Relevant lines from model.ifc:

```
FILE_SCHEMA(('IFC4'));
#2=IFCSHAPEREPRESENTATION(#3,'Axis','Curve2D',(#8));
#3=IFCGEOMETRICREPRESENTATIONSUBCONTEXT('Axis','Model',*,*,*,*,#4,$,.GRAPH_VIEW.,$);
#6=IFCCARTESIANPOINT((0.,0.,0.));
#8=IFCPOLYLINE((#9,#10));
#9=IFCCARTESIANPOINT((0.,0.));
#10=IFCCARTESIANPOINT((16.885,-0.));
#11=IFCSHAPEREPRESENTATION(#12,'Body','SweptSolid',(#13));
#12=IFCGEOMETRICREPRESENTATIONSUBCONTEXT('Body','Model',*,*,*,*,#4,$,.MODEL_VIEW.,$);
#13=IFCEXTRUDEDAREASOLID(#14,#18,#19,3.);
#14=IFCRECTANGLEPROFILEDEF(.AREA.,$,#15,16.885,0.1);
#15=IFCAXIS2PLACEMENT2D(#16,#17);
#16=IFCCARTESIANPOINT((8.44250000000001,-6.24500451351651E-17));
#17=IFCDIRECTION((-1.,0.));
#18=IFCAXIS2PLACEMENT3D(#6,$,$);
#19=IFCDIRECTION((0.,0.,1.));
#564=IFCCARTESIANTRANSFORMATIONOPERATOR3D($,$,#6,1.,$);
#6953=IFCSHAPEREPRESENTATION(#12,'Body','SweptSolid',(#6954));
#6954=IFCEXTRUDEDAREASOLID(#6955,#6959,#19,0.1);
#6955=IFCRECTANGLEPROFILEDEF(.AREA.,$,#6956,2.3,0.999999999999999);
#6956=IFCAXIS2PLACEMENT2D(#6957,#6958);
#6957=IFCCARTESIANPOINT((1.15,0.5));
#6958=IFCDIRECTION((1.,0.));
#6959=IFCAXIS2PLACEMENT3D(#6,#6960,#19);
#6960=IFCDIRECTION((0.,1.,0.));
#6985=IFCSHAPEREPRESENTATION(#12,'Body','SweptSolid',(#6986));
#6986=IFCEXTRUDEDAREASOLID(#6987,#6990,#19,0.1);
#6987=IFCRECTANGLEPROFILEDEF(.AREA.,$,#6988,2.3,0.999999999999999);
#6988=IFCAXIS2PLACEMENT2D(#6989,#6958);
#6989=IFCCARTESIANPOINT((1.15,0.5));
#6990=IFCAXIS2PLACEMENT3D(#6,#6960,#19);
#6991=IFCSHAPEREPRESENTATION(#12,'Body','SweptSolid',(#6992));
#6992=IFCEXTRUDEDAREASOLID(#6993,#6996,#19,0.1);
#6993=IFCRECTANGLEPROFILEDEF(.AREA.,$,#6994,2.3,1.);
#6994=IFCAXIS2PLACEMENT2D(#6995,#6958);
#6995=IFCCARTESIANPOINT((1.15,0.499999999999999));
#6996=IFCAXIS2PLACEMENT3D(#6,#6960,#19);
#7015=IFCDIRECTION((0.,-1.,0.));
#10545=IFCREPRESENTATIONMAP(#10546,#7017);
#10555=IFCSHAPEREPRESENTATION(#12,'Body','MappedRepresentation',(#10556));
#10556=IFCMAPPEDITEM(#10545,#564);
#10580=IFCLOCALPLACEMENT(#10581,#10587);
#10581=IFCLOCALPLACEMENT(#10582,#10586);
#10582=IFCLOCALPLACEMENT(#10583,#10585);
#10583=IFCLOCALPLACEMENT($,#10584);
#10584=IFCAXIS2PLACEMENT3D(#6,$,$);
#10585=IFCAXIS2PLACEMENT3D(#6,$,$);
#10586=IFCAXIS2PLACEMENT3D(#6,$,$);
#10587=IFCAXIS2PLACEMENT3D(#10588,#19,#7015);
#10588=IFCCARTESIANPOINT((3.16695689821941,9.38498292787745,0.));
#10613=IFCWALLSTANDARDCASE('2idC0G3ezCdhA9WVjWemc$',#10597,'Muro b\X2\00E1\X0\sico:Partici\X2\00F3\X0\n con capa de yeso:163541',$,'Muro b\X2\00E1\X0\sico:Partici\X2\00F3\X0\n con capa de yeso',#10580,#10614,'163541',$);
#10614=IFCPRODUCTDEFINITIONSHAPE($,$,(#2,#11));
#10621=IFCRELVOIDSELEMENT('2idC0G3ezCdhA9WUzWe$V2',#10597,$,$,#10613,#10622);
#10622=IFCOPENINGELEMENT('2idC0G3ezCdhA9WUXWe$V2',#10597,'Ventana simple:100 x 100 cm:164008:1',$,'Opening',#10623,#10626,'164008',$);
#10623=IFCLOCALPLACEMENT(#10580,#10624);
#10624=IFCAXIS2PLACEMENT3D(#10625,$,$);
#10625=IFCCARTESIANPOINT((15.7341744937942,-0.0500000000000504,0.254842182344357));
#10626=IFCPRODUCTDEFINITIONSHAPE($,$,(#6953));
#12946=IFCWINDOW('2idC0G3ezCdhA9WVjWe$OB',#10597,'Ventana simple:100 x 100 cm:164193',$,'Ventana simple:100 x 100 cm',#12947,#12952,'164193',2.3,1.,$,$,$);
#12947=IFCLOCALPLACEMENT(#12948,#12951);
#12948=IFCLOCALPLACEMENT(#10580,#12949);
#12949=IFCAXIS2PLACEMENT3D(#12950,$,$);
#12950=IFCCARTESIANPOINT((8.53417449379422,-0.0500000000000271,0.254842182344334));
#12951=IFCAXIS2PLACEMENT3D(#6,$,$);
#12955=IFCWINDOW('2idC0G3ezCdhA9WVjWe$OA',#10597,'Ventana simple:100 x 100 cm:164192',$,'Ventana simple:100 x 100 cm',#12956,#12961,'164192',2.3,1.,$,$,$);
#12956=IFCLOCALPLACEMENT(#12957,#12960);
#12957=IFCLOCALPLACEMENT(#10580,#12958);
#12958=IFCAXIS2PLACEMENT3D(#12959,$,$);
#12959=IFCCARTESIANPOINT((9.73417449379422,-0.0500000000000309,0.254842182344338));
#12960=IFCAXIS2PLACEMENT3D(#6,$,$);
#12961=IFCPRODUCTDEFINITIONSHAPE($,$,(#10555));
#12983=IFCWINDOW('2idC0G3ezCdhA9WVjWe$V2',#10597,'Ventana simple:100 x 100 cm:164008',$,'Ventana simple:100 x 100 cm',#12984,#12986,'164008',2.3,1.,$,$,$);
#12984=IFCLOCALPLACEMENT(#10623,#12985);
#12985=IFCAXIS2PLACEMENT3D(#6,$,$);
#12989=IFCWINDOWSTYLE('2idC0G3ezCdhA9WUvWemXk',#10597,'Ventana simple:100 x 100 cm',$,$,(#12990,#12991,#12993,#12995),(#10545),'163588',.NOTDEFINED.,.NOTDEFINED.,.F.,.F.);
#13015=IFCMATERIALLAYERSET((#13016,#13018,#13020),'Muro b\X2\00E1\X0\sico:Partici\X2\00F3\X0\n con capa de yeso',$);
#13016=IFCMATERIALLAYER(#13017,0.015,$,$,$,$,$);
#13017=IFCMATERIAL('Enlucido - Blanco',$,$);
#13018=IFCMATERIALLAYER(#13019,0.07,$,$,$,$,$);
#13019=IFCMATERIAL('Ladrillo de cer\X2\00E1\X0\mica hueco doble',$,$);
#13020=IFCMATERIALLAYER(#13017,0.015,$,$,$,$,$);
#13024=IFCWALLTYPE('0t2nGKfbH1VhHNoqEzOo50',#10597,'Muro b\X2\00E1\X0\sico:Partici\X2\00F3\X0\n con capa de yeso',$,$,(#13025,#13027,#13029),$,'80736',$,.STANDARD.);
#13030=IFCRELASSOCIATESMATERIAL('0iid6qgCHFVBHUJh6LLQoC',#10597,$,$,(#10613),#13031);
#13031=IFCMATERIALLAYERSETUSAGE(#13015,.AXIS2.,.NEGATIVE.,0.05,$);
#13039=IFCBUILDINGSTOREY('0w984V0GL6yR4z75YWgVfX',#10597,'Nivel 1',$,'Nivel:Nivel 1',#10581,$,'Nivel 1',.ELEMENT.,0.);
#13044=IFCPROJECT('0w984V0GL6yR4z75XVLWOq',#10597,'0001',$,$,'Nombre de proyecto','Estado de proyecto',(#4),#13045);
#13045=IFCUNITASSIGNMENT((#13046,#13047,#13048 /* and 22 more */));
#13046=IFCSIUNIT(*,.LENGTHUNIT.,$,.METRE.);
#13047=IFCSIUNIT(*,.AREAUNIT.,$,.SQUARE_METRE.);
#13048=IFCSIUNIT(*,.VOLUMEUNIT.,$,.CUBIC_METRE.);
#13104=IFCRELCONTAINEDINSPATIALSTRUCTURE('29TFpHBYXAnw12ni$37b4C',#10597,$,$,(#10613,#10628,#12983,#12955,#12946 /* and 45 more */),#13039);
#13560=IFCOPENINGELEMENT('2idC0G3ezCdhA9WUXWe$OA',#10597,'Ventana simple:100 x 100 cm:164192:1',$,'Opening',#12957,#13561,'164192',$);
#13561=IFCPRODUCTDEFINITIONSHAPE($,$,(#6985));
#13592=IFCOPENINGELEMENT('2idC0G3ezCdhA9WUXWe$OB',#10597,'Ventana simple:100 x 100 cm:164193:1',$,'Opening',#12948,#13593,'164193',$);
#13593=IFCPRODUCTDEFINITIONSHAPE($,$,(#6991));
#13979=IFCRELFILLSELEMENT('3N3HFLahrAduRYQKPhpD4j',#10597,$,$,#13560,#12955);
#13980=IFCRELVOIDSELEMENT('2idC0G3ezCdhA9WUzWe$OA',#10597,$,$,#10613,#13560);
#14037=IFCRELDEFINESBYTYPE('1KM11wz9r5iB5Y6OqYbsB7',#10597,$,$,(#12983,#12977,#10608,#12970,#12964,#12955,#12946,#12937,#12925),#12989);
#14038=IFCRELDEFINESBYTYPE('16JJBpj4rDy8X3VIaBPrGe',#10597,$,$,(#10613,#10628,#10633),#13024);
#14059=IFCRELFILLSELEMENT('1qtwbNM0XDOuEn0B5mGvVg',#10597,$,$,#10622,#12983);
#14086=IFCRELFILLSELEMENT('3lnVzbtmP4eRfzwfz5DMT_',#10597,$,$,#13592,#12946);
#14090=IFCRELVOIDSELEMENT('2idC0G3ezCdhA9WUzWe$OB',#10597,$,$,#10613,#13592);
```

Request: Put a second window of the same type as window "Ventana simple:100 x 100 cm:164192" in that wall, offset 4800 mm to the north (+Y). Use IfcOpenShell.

```python
import ifcopenshell
import ifcopenshell.api.feature
import ifcopenshell.api.geometry
import ifcopenshell.api.root
import ifcopenshell.geom
import ifcopenshell.util.element
import ifcopenshell.util.placement
import ifcopenshell.util.shape

model = ifcopenshell.open("model.ifc")
settings = ifcopenshell.geom.settings()


def volume(element):
    """Net volume in cubic metres, openings subtracted."""
    shape = ifcopenshell.geom.create_shape(settings, element)
    return ifcopenshell.util.shape.get_volume(shape.geometry)


def reuse_history(source, copy):
    """copy_class also copies each property set's owner history, people and application; keep the originals."""
    for rel in copy.IsDefinedBy:
        if rel.is_a("IfcRelDefinesByProperties") and (history := rel.RelatingPropertyDefinition.OwnerHistory):
            rel.RelatingPropertyDefinition.OwnerHistory = source.OwnerHistory
            ifcopenshell.util.element.remove_deep2(model, history)


window = model.by_guid("2idC0G3ezCdhA9WVjWe$OA")
opening = window.FillsVoids[0].RelatingOpeningElement
wall = opening.VoidsElements[0].RelatingBuildingElement
before = volume(wall)
shift = ifcopenshell.util.placement.get_local_placement(wall.ObjectPlacement)[:3, 0] * -4.8

# copy_class copies the void relationship, type, container and properties, but no geometry.
new_opening = ifcopenshell.api.root.copy_class(model, product=opening)
new_opening.Representation = ifcopenshell.util.element.copy_deep(
    model, opening.Representation, exclude=["IfcGeometricRepresentationContext", "IfcRepresentationMap"]
)
new_opening.Name = "Ventana simple:100 x 100 cm"
new_opening.Tag = None
new_window = ifcopenshell.api.root.copy_class(model, product=window)
new_window.Representation = ifcopenshell.util.element.copy_deep(
    model, window.Representation, exclude=["IfcGeometricRepresentationContext", "IfcRepresentationMap"]
)
new_window.Name = "Ventana simple:100 x 100 cm"
new_window.Tag = None
reuse_history(window, new_window)
ifcopenshell.api.feature.add_filling(model, opening=new_opening, element=new_window)

for old, new in ((opening, new_opening), (window, new_window)):
    matrix = ifcopenshell.util.placement.get_local_placement(old.ObjectPlacement)
    matrix[:3, 3] += shift
    ifcopenshell.api.geometry.edit_object_placement(model, product=new, matrix=matrix, is_si=False)

after = volume(wall)

print(f"wall volume {before:.3f} -> {after:.3f} m3")

model.write("model_v2.ifc")
```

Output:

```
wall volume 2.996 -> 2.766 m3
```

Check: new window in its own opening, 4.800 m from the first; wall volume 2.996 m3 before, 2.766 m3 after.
